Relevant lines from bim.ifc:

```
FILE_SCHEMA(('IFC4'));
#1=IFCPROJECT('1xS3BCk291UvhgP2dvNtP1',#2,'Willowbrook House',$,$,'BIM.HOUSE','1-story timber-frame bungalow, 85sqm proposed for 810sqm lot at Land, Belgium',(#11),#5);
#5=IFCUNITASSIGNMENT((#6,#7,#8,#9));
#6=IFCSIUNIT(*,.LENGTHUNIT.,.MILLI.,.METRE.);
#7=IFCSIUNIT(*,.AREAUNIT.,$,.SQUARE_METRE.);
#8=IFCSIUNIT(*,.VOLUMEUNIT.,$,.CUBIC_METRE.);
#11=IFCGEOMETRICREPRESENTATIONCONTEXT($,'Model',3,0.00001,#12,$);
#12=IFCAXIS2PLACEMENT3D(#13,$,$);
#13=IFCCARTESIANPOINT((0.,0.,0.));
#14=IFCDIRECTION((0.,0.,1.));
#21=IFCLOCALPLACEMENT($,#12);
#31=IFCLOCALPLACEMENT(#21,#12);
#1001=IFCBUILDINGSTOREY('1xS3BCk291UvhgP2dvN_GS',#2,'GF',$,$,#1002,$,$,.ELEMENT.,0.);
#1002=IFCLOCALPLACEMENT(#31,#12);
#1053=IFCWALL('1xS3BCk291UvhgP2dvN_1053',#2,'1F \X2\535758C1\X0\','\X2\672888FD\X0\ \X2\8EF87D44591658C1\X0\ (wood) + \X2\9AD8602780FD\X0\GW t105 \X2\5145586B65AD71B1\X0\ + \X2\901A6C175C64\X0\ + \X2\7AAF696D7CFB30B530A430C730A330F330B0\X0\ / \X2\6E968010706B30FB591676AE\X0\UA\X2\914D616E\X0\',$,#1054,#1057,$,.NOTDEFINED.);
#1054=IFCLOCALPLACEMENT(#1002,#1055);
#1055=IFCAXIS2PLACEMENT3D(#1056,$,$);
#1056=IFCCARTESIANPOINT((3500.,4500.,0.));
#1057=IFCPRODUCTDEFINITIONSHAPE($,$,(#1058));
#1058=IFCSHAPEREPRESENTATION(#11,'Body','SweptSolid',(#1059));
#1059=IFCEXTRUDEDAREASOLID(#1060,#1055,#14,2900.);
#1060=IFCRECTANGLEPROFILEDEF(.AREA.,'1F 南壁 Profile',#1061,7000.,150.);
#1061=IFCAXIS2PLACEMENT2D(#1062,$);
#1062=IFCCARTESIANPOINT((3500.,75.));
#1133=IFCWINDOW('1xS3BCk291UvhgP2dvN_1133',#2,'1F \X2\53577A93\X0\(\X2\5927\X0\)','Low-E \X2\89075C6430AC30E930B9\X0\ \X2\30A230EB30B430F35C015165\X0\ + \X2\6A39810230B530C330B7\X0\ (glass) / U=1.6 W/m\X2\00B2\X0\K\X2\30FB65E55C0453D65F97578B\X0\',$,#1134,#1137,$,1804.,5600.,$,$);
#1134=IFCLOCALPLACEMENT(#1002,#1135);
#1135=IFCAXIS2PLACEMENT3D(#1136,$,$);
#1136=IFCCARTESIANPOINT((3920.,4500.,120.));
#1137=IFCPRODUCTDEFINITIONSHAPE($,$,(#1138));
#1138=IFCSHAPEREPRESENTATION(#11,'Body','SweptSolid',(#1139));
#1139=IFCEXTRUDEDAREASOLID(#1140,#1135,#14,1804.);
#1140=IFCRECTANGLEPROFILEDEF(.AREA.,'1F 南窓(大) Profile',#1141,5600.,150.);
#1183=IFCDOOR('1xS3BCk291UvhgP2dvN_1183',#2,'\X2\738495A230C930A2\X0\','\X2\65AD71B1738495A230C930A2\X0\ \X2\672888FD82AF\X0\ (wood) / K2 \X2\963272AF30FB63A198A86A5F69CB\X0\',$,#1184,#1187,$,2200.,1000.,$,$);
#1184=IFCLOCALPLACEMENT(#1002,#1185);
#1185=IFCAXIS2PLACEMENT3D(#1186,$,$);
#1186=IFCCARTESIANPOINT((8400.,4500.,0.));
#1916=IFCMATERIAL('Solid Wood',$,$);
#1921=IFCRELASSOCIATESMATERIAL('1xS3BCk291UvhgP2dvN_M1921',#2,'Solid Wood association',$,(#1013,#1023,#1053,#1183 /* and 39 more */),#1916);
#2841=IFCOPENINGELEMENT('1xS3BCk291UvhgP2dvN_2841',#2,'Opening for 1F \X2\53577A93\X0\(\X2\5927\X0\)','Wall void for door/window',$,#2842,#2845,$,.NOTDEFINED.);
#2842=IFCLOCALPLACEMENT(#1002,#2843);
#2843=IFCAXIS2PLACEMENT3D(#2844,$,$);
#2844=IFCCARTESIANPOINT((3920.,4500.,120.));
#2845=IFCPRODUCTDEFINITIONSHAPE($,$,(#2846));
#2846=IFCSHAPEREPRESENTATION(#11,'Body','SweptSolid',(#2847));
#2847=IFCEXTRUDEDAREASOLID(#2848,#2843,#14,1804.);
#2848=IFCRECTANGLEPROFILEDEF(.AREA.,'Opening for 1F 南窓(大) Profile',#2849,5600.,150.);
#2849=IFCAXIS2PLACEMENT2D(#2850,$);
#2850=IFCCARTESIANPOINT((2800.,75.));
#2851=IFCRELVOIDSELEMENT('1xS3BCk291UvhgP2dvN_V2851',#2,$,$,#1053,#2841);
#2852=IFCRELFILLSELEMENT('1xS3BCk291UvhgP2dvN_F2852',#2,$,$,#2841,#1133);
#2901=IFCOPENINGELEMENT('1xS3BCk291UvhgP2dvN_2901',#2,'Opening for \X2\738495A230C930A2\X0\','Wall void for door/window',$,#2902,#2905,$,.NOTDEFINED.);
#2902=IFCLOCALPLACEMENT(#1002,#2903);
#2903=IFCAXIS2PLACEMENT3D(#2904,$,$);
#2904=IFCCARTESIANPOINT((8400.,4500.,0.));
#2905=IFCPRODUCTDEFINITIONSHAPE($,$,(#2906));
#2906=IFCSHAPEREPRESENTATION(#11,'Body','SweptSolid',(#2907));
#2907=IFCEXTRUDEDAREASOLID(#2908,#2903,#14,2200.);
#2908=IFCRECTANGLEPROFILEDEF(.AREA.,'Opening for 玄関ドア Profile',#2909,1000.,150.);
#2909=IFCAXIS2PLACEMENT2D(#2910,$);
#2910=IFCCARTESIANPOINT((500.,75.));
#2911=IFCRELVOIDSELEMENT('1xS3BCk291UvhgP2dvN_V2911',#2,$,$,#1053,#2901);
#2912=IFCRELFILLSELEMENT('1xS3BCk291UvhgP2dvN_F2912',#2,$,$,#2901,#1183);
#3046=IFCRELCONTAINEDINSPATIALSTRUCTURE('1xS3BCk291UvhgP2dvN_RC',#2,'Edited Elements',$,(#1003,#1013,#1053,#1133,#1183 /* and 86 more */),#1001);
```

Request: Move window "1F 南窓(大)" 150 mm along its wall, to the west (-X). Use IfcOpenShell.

```python
import ifcopenshell
import ifcopenshell.api.geometry
import ifcopenshell.util.placement
import ifcopenshell.util.unit

model = ifcopenshell.open("bim.ifc")
unit_scale = ifcopenshell.util.unit.calculate_unit_scale(model)

window = model.by_id(1133)
opening = window.FillsVoids[0].RelatingOpeningElement
wall = opening.VoidsElements[0].RelatingBuildingElement

wall_matrix = ifcopenshell.util.placement.get_local_placement(wall.ObjectPlacement)
shift = wall_matrix[:3, 0] * -0.15 / unit_scale
before = ifcopenshell.util.placement.get_local_placement(window.ObjectPlacement)[:3, 3].copy()

# The window is not placed relative to its opening, so move both.
for product in (opening, window):
    matrix = ifcopenshell.util.placement.get_local_placement(product.ObjectPlacement)
    matrix[:3, 3] += shift
    ifcopenshell.api.geometry.edit_object_placement(model, product=product, matrix=matrix, is_si=False)

after = ifcopenshell.util.placement.get_local_placement(window.ObjectPlacement)[:3, 3]
print("window moved by", (after - before).round(3) + 0.0)

model.write("bim_updated.ifc")
```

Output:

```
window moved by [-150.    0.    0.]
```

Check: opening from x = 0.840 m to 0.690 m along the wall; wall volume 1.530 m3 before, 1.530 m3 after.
